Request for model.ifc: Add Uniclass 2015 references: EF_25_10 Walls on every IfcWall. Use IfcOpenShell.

First a look at what the model holds.

```python
import ifcopenshell

model = ifcopenshell.open("model.ifc")
print(model.schema)
print("classifications:", [c.Name for c in model.by_type("IfcClassification")])
for ifc_class in ("IfcDoor", "IfcRoof", "IfcStair", "IfcWall", "IfcWindow"):
    print(ifc_class, len(model.by_type(ifc_class)))
```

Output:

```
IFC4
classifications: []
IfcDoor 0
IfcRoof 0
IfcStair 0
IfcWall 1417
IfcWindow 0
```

```python
import ifcopenshell
import ifcopenshell.api.classification

model = ifcopenshell.open("model.ifc")

system = ifcopenshell.api.classification.add_classification(model, classification="Uniclass 2015")

codes = {
    "IfcWall": ("EF_25_10", "Walls"),
}
for ifc_class, (code, name) in codes.items():
    products = model.by_type(ifc_class)
    ifcopenshell.api.classification.add_reference(
        model, products=products, classification=system, identification=code, name=name
    )
    print(code, len(products))

model.write("model-out.ifc")
```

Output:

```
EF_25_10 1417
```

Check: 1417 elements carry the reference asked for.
